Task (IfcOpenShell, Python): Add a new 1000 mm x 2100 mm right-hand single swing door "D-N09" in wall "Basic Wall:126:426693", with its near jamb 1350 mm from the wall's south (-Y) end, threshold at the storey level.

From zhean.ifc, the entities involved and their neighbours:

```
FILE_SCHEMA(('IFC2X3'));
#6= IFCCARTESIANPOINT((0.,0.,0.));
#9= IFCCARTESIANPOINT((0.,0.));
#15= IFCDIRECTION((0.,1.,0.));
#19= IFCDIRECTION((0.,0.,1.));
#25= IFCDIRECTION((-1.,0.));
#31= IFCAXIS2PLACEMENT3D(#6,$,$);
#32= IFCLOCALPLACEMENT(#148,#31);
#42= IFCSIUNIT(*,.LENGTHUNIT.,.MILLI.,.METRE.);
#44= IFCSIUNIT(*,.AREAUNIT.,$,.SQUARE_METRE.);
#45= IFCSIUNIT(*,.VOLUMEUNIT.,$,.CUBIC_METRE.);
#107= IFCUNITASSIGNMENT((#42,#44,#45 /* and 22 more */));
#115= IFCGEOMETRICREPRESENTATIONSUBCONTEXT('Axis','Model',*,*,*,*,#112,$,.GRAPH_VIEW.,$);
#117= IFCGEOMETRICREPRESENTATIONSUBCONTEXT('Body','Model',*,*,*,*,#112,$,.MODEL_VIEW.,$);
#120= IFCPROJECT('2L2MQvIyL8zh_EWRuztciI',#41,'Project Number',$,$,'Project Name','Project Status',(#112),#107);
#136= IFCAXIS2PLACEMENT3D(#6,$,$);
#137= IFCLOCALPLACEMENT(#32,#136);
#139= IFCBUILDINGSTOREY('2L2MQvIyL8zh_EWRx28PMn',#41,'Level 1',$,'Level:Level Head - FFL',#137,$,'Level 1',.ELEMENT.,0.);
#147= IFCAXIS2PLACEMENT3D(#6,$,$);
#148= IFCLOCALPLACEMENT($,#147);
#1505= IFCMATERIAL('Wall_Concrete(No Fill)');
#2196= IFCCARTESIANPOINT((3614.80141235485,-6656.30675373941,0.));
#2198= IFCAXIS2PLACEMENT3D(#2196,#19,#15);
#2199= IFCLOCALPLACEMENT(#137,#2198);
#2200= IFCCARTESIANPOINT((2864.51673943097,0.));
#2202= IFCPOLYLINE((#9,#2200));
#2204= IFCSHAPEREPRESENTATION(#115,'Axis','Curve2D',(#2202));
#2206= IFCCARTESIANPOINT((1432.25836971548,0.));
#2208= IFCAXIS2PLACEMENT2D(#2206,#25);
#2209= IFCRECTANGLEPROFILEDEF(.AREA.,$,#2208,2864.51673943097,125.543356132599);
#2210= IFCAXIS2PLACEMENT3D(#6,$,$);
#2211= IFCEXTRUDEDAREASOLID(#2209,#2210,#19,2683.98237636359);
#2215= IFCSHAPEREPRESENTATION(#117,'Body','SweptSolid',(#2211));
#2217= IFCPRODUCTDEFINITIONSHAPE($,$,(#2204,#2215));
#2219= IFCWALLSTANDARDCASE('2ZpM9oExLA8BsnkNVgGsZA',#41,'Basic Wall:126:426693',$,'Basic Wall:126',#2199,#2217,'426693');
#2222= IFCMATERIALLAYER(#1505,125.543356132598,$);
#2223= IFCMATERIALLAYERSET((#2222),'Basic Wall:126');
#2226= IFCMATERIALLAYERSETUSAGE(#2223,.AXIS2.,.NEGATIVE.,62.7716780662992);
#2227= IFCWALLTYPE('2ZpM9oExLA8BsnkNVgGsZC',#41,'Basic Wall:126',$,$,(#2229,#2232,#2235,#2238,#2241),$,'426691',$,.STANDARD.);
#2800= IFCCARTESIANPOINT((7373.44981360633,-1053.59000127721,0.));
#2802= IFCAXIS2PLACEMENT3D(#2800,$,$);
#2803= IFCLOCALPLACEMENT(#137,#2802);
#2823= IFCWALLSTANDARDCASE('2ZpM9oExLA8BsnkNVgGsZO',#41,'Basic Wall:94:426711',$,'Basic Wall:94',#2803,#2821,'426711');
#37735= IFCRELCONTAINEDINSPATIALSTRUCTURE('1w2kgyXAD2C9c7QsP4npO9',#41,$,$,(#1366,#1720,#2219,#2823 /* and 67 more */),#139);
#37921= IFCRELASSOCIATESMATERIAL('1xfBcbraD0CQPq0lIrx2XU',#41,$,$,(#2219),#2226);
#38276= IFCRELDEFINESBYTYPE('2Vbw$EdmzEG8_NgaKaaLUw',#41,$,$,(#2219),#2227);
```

```python
import numpy as np
import ifcopenshell
import ifcopenshell.api.feature
import ifcopenshell.api.geometry
import ifcopenshell.api.root
import ifcopenshell.api.spatial
import ifcopenshell.api.type
import ifcopenshell.geom
import ifcopenshell.util.element
import ifcopenshell.util.placement
import ifcopenshell.util.representation
import ifcopenshell.util.shape
import ifcopenshell.util.unit

model = ifcopenshell.open("zhean.ifc")
unit_scale = ifcopenshell.util.unit.calculate_unit_scale(model)
settings = ifcopenshell.geom.settings()


def volume(element):
    """Net volume in cubic metres, openings subtracted."""
    shape = ifcopenshell.geom.create_shape(settings, element)
    return ifcopenshell.util.shape.get_volume(shape.geometry)


wall = model.by_guid("2ZpM9oExLA8BsnkNVgGsZA")
storey = ifcopenshell.util.element.get_container(wall, ifc_class="IfcBuildingStorey")
context = ifcopenshell.util.representation.get_context(model, "Model", "Body", "MODEL_VIEW")
before = volume(wall)

width, height, from_end, sill = 1, 2.1, 1.35, 0.0  # metres

# The wall runs along its own X axis, and the end named is its -X end.
wall_shape = ifcopenshell.geom.create_shape(settings, wall)
x, y, z = ifcopenshell.util.shape.get_vertices(wall_shape.geometry).T
start = x.min() + from_end
face, thickness = float(y.min()), float(y.max() - y.min())
wall_matrix = ifcopenshell.util.placement.get_local_placement(wall.ObjectPlacement)
level = ifcopenshell.util.placement.get_local_placement(storey.ObjectPlacement)[2, 3]


def in_wall(x, y):
    """Placement at x, y metres in the wall's axes, at sill height."""
    matrix = wall_matrix.copy()
    matrix[:, 3] = wall_matrix @ np.array([x / unit_scale, y / unit_scale, 0.0, 1.0])
    matrix[2, 3] = level + sill / unit_scale
    return matrix


# Opening: a box that overshoots both wall faces by 50 mm.
opening = ifcopenshell.api.root.create_entity(model, ifc_class="IfcOpeningElement")
box = ifcopenshell.api.geometry.add_wall_representation(
    model, context=context, length=width, height=height, thickness=thickness + 0.1
)
ifcopenshell.api.geometry.assign_representation(model, product=opening, representation=box)
ifcopenshell.api.geometry.edit_object_placement(model, product=opening, matrix=in_wall(start, face - 0.05), is_si=False)
ifcopenshell.api.feature.add_feature(model, feature=opening, element=wall)

door = ifcopenshell.api.root.create_entity(model, ifc_class="IfcDoor", name="D-N09")
door.OverallWidth, door.OverallHeight = width / unit_scale, height / unit_scale
body = ifcopenshell.api.geometry.add_door_representation(
    model,
    context=context,
    overall_width=door.OverallWidth,
    overall_height=door.OverallHeight,
    operation_type="SINGLE_SWING_RIGHT",
    lining_properties={"LiningDepth": thickness / unit_scale, "ThresholdDepth": thickness / unit_scale},
)
ifcopenshell.api.geometry.assign_representation(model, product=door, representation=body)
ifcopenshell.api.spatial.assign_container(model, products=[door], relating_structure=storey)
fills = ifcopenshell.api.feature.add_filling(model, opening=opening, element=door)
fills.OwnerHistory = door.OwnerHistory  # required in IFC2X3

# IFC2X3 keeps the operation on the door style.
style = ifcopenshell.api.root.create_entity(model, ifc_class="IfcDoorStyle", name="D-N09")
style.OperationType, style.ConstructionType = "SINGLE_SWING_RIGHT", "NOTDEFINED"
style.ParameterTakesPrecedence = style.Sizeable = False
ifcopenshell.api.type.assign_type(model, related_objects=[door], relating_type=style)

# The lining spans the wall, so the door starts at the wall face.
ifcopenshell.api.geometry.edit_object_placement(model, product=door, matrix=in_wall(start, face), is_si=False)

after = volume(wall)

print(f"wall volume {before:.3f} -> {after:.3f} m3")

model.write("zhean-out.ifc")
```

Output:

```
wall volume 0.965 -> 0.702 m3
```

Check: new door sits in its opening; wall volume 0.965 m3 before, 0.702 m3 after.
